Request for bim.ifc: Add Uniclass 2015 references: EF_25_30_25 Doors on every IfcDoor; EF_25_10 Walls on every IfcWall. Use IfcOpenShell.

First a look at what the model holds.

```python
import ifcopenshell

model = ifcopenshell.open("bim.ifc")
print(model.schema)
print("classifications:", [c.Name for c in model.by_type("IfcClassification")])
for ifc_class in ("IfcDoor", "IfcRoof", "IfcStair", "IfcWall", "IfcWindow"):
    print(ifc_class, len(model.by_type(ifc_class)))
```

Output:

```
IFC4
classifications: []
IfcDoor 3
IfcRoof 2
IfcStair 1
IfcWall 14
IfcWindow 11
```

```python
import ifcopenshell
import ifcopenshell.api.classification

model = ifcopenshell.open("bim.ifc")

system = ifcopenshell.api.classification.add_classification(model, classification="Uniclass 2015")

codes = {
    "IfcDoor": ("EF_25_30_25", "Doors"),
    "IfcWall": ("EF_25_10", "Walls"),
}
for ifc_class, (code, name) in codes.items():
    products = model.by_type(ifc_class)
    ifcopenshell.api.classification.add_reference(
        model, products=products, classification=system, identification=code, name=name
    )
    print(code, len(products))

model.write("bim-out.ifc")
```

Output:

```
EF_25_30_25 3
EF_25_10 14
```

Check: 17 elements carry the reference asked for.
